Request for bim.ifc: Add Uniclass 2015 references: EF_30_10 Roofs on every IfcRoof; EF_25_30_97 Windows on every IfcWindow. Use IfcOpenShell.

First a look at what the model holds.

```python
import ifcopenshell

model = ifcopenshell.open("bim.ifc")
print(model.schema)
print("classifications:", [c.Name for c in model.by_type("IfcClassification")])
for ifc_class in ("IfcDoor", "IfcRoof", "IfcStair", "IfcWall", "IfcWindow"):
    print(ifc_class, len(model.by_type(ifc_class)))
```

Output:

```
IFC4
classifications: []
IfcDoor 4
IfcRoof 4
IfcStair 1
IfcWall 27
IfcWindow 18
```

```python
import ifcopenshell
import ifcopenshell.api.classification

model = ifcopenshell.open("bim.ifc")

system = ifcopenshell.api.classification.add_classification(model, classification="Uniclass 2015")

codes = {
    "IfcRoof": ("EF_30_10", "Roofs"),
    "IfcWindow": ("EF_25_30_97", "Windows"),
}
for ifc_class, (code, name) in codes.items():
    products = model.by_type(ifc_class)
    ifcopenshell.api.classification.add_reference(
        model, products=products, classification=system, identification=code, name=name
    )
    print(code, len(products))

model.write("bim-out.ifc")
```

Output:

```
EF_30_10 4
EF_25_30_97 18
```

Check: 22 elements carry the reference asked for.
